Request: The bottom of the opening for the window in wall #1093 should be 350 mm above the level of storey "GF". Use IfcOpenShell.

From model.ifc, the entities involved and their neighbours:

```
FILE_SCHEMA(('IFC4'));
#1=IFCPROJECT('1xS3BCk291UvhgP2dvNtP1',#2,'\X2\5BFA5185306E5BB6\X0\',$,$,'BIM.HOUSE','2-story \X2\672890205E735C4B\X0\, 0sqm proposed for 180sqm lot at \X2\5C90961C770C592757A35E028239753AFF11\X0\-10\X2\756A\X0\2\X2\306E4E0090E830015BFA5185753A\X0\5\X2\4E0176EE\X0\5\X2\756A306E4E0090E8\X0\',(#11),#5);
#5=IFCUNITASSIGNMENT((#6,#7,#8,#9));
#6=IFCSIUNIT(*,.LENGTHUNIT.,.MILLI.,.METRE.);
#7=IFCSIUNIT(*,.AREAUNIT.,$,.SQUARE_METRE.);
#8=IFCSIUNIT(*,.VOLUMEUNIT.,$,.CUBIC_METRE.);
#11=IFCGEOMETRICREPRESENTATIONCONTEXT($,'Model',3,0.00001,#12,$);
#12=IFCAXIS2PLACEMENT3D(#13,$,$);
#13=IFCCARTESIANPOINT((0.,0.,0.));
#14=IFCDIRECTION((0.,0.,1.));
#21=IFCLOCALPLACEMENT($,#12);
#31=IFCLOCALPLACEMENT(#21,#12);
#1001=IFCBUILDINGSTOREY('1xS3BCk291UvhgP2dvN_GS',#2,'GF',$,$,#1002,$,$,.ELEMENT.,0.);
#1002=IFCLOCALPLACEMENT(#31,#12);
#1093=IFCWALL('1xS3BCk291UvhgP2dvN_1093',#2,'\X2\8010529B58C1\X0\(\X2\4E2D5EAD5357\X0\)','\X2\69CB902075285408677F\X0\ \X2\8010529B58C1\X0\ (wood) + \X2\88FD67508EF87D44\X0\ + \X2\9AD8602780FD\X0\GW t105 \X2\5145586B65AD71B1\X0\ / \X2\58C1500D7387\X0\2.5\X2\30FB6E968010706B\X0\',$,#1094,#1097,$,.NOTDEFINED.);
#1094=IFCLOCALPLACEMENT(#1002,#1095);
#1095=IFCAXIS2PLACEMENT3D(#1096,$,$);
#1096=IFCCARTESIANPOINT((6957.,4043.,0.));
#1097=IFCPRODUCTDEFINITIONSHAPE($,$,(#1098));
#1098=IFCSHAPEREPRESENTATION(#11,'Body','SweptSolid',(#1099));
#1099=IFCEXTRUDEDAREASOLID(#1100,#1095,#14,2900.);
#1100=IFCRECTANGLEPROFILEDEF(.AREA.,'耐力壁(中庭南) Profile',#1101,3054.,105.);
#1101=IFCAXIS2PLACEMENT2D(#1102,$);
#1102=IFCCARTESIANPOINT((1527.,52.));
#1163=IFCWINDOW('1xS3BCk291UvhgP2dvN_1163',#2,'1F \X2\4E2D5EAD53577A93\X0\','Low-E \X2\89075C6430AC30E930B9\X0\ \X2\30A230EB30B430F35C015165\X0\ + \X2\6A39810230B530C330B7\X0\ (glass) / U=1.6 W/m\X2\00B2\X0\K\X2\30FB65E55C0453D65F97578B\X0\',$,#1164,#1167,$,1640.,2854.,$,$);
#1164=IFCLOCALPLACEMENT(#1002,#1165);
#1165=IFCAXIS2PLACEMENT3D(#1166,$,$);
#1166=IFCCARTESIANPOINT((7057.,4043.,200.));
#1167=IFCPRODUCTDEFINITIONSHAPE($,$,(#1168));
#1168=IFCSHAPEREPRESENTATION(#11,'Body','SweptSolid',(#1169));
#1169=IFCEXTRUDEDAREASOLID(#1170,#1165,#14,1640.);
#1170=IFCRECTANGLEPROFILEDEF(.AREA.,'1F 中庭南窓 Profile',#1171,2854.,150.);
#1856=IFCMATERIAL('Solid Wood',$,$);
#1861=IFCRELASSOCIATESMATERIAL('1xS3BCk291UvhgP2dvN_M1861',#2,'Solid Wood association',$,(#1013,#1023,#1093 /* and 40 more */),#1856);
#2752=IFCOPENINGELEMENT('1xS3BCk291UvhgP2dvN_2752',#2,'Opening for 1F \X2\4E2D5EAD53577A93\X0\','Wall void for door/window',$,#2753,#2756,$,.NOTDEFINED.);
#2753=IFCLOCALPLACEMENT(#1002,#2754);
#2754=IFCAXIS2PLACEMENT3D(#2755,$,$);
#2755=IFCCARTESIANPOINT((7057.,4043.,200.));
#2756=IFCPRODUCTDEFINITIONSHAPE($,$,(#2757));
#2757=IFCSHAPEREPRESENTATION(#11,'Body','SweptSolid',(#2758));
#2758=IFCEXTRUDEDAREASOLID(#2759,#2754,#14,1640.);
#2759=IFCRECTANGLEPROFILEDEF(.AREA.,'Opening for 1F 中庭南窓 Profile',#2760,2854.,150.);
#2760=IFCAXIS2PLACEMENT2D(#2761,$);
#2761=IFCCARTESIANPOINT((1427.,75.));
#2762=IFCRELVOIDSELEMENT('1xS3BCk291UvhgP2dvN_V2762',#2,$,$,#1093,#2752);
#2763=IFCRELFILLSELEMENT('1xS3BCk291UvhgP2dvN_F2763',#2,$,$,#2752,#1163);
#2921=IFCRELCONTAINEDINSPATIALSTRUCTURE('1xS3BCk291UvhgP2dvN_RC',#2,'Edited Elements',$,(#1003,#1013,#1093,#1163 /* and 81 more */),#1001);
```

```python
import numpy as np
import ifcopenshell
import ifcopenshell.api.geometry
import ifcopenshell.geom
import ifcopenshell.util.element
import ifcopenshell.util.placement
import ifcopenshell.util.shape
import ifcopenshell.util.unit

model = ifcopenshell.open("model.ifc")
unit_scale = ifcopenshell.util.unit.calculate_unit_scale(model)

window = model.by_id(1163)
opening = window.FillsVoids[0].RelatingOpeningElement
storey = ifcopenshell.util.element.get_container(window, ifc_class="IfcBuildingStorey")
level = ifcopenshell.util.placement.get_local_placement(storey.ObjectPlacement)[2, 3]

# The opening's origin need not be at the sill, so measure its lowest point.
shape = ifcopenshell.geom.create_shape(ifcopenshell.geom.settings(), opening)
bottom = ifcopenshell.util.shape.get_shape_bottom_elevation(shape, shape.geometry) / unit_scale
dz = level + 0.35 / unit_scale - bottom

shift = np.array([0.0, 0.0, dz])
# The window is not placed relative to its opening, so move both.
for product in (opening, window):
    matrix = ifcopenshell.util.placement.get_local_placement(product.ObjectPlacement)
    matrix[:3, 3] += shift
    ifcopenshell.api.geometry.edit_object_placement(model, product=product, matrix=matrix, is_si=False)

print(f"moved by {dz * unit_scale:+.3f} m")

model.write("model_updated.ifc")
```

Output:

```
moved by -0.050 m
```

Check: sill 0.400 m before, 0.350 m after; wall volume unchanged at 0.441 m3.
